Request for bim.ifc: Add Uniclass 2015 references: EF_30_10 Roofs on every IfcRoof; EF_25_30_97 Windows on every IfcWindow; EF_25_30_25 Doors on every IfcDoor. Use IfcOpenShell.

First a look at what the model holds.

```python
import ifcopenshell

model = ifcopenshell.open("bim.ifc")
print(model.schema)
print("classifications:", [c.Name for c in model.by_type("IfcClassification")])
for ifc_class in ("IfcDoor", "IfcRoof", "IfcStair", "IfcWall", "IfcWindow"):
    print(ifc_class, len(model.by_type(ifc_class)))
```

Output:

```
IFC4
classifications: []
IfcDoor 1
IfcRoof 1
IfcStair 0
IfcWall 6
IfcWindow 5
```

```python
import ifcopenshell
import ifcopenshell.api.classification

model = ifcopenshell.open("bim.ifc")

system = ifcopenshell.api.classification.add_classification(model, classification="Uniclass 2015")

codes = {
    "IfcRoof": ("EF_30_10", "Roofs"),
    "IfcWindow": ("EF_25_30_97", "Windows"),
    "IfcDoor": ("EF_25_30_25", "Doors"),
}
for ifc_class, (code, name) in codes.items():
    products = model.by_type(ifc_class)
    ifcopenshell.api.classification.add_reference(
        model, products=products, classification=system, identification=code, name=name
    )
    print(code, len(products))

model.write("bim_updated.ifc")
```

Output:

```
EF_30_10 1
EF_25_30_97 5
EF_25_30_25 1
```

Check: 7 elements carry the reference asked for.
